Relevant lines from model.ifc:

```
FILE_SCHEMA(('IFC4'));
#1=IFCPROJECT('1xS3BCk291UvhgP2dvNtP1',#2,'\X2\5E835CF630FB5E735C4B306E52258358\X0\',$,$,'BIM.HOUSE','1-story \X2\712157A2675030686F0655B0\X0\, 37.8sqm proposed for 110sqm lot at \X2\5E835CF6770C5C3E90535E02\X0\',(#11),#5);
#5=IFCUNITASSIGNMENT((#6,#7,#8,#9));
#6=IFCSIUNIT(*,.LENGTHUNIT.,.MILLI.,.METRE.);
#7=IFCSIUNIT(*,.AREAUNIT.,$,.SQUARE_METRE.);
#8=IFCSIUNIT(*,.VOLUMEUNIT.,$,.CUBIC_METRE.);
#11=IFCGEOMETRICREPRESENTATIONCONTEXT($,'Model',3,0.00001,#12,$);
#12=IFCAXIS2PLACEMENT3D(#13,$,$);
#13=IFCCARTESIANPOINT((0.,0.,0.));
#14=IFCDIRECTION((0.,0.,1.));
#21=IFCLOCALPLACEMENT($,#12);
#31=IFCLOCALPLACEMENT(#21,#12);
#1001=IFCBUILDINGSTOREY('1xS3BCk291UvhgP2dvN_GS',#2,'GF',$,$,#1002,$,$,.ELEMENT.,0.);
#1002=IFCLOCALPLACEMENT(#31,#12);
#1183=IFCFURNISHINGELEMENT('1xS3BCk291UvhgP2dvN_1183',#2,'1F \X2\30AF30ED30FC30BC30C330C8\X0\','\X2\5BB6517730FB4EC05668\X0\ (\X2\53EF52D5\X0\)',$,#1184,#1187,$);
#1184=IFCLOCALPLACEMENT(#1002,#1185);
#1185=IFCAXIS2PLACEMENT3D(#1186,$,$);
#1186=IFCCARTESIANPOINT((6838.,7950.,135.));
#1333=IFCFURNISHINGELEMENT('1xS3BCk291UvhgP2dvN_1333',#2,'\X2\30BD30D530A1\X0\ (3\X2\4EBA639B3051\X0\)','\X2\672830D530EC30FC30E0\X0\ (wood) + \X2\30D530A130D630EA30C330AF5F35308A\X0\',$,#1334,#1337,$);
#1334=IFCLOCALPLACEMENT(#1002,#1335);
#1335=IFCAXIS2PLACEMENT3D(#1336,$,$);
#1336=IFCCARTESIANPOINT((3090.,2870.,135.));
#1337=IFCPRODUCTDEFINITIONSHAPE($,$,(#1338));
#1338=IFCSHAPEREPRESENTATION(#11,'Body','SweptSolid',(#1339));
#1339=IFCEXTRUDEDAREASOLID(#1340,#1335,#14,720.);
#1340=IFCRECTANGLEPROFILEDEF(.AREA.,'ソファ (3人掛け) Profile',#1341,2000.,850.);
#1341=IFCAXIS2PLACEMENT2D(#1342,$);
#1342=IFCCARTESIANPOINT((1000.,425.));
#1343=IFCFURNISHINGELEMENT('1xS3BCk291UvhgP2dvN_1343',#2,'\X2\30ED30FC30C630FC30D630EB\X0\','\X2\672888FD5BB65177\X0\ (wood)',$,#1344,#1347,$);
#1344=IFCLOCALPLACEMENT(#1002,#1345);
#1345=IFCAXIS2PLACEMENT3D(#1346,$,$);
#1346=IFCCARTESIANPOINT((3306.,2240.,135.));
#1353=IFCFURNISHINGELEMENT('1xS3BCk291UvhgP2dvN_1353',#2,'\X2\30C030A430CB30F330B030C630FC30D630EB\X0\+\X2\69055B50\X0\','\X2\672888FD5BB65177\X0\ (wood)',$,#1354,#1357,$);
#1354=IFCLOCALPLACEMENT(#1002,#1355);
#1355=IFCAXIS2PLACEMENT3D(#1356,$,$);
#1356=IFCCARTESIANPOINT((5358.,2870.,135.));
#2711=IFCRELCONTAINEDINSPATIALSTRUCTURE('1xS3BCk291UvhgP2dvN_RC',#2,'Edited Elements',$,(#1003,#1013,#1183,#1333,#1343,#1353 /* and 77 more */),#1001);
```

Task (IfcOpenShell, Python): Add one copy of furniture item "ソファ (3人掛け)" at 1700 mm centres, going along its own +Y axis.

```python
import ifcopenshell
import ifcopenshell.api.geometry
import ifcopenshell.api.root
import ifcopenshell.util.element
import ifcopenshell.util.placement
import ifcopenshell.util.unit

model = ifcopenshell.open("model.ifc")
unit_scale = ifcopenshell.util.unit.calculate_unit_scale(model)


def reuse_history(source, copy):
    """copy_class also copies each property set's owner history, people and application; keep the originals."""
    for rel in copy.IsDefinedBy:
        if rel.is_a("IfcRelDefinesByProperties") and (history := rel.RelatingPropertyDefinition.OwnerHistory):
            rel.RelatingPropertyDefinition.OwnerHistory = source.OwnerHistory
            ifcopenshell.util.element.remove_deep2(model, history)


source = model.by_id(1333)
base = ifcopenshell.util.placement.get_local_placement(source.ObjectPlacement)
step = base[:3, 1] * 1.7 / unit_scale

for i in range(1, 2):
    copy = ifcopenshell.api.root.copy_class(model, product=source)
    copy.Representation = ifcopenshell.util.element.copy_deep(
        model, source.Representation, exclude=["IfcGeometricRepresentationContext", "IfcRepresentationMap"]
    )
    reuse_history(source, copy)
    matrix = base.copy()
    matrix[:3, 3] += i * step
    print("added at", matrix[:3, 3].round(3) + 0.0)
    ifcopenshell.api.geometry.edit_object_placement(model, product=copy, matrix=matrix, is_si=False)

model.write("model-out.ifc")
```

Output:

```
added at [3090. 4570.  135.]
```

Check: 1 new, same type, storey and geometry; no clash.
